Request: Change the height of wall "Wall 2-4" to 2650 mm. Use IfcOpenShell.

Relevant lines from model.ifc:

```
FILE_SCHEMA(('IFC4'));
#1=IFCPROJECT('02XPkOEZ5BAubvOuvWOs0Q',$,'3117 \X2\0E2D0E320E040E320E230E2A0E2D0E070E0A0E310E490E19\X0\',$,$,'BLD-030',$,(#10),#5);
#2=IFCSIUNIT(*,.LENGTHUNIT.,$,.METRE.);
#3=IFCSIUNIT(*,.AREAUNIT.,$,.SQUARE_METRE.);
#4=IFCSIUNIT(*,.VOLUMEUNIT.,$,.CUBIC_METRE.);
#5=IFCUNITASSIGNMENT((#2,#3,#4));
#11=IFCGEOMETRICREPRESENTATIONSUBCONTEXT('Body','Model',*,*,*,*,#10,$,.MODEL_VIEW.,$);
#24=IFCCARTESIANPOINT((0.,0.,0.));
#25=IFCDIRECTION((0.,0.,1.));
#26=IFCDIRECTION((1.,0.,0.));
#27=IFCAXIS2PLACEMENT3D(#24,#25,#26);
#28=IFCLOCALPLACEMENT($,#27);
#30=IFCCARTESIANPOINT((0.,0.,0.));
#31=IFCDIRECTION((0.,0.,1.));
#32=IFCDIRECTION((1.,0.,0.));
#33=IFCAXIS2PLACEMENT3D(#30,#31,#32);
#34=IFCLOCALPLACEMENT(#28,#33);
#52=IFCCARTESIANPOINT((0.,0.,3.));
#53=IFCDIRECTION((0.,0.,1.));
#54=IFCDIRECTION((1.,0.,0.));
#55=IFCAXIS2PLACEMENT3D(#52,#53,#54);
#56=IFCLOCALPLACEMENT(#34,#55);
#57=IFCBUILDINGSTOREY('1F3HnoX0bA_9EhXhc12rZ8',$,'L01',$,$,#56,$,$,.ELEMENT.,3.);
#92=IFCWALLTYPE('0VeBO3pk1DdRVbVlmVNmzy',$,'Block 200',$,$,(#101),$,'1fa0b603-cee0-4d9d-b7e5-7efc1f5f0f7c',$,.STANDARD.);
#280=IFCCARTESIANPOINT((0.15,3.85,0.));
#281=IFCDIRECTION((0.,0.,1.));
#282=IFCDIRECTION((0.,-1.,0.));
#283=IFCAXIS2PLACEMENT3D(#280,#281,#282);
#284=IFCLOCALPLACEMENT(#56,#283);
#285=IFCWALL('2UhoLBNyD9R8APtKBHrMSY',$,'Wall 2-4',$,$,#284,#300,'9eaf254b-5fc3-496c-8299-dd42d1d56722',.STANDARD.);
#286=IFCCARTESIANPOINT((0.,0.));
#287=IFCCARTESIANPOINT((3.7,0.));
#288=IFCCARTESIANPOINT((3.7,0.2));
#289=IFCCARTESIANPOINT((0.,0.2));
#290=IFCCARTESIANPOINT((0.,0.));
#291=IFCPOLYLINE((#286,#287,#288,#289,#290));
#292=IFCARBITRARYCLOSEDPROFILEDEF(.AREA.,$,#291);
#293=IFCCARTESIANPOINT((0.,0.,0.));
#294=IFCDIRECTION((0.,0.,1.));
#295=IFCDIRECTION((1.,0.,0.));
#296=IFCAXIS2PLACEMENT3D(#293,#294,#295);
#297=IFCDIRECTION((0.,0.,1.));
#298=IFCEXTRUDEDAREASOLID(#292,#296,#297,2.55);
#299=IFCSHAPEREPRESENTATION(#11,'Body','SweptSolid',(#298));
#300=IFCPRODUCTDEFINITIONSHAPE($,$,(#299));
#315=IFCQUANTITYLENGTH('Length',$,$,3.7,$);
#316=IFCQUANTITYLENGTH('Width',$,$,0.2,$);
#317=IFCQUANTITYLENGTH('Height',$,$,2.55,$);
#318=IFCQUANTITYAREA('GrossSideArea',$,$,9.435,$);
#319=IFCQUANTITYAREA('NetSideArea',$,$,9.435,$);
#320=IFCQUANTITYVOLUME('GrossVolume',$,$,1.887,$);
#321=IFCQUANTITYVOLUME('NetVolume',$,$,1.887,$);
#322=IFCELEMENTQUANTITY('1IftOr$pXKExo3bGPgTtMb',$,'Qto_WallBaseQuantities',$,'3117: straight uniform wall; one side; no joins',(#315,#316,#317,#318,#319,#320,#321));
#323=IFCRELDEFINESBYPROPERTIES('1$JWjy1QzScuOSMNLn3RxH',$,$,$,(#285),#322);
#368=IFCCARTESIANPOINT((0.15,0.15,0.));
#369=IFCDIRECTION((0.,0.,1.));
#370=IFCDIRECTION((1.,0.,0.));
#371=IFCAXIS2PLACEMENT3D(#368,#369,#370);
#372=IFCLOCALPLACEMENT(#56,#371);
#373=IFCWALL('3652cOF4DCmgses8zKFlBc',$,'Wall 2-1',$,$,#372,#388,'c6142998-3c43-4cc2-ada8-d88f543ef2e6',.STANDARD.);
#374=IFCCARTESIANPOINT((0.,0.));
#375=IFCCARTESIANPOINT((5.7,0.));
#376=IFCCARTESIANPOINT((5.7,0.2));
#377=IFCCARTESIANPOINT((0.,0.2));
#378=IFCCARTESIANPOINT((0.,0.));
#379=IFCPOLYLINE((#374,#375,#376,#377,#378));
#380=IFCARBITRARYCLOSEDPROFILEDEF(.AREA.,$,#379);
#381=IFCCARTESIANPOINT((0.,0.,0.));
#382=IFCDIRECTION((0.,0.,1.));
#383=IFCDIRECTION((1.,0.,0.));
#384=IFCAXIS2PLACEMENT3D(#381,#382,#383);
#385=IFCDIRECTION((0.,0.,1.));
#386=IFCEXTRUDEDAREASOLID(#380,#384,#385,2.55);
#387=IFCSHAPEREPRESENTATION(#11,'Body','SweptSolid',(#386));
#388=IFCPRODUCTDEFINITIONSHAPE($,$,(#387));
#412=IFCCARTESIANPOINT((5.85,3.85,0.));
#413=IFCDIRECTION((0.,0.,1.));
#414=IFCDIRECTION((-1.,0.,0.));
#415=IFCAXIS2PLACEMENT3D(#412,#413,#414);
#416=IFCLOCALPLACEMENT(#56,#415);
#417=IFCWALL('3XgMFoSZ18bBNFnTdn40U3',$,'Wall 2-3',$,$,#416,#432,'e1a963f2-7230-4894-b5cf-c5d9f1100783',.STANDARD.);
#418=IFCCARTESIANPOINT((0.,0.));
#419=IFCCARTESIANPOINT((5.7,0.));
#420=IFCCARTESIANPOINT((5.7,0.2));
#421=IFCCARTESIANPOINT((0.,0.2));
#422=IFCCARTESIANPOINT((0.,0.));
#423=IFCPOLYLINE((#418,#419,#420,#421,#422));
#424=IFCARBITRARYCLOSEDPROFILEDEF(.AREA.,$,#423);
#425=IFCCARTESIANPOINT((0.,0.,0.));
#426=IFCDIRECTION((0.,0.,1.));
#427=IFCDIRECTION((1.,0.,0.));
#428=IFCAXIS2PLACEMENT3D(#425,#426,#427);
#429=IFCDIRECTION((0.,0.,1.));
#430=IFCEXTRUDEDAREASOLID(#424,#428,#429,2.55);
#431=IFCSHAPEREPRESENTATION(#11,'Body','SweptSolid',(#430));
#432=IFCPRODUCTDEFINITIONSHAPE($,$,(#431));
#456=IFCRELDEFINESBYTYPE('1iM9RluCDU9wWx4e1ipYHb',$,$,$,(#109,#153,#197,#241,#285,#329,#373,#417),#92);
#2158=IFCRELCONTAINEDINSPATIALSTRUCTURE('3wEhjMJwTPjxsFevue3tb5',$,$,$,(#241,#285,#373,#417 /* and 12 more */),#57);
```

```python
import ifcopenshell
import ifcopenshell.api.pset
import ifcopenshell.geom
import ifcopenshell.util.element
import ifcopenshell.util.representation
import ifcopenshell.util.shape
import ifcopenshell.util.unit

model = ifcopenshell.open("model.ifc")
unit_scale = ifcopenshell.util.unit.calculate_unit_scale(model)
area_scale = ifcopenshell.util.unit.calculate_unit_scale(model, "AREAUNIT")
volume_scale = ifcopenshell.util.unit.calculate_unit_scale(model, "VOLUMEUNIT")
settings = ifcopenshell.geom.settings()


def volume(element):
    """Net volume in cubic metres, openings subtracted."""
    shape = ifcopenshell.geom.create_shape(settings, element)
    return ifcopenshell.util.shape.get_volume(shape.geometry)


wall = model.by_guid("2UhoLBNyD9R8APtKBHrMSY")
before = volume(wall)

body = ifcopenshell.util.representation.get_representation(wall, "Model", "Body")
solid = body.Items[0]
old_height = solid.Depth
solid.Depth = 2.65 / unit_scale
after = volume(wall)
thickness = 0.2  # wall thickness in metres

# Update the stored height, areas and volumes.
qto = model.by_id(ifcopenshell.util.element.get_pset(wall, "Qto_WallBaseQuantities", should_inherit=False)["id"])
ifcopenshell.api.pset.edit_qto(model, qto=qto, properties={
    "Height": solid.Depth,
    "GrossSideArea": ifcopenshell.util.element.get_pset(wall, "Qto_WallBaseQuantities", "GrossSideArea") * solid.Depth / old_height,
    "NetSideArea": after / thickness / area_scale,
    "GrossVolume": ifcopenshell.util.element.get_pset(wall, "Qto_WallBaseQuantities", "GrossVolume") * solid.Depth / old_height,
    "NetVolume": after / volume_scale,
})

print(f"height {old_height:g} -> {solid.Depth:g}, volume {before:.3f} -> {after:.3f} m3")

model.write("model_edited.ifc")
```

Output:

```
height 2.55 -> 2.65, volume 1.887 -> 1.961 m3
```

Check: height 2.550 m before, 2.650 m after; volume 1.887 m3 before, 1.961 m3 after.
